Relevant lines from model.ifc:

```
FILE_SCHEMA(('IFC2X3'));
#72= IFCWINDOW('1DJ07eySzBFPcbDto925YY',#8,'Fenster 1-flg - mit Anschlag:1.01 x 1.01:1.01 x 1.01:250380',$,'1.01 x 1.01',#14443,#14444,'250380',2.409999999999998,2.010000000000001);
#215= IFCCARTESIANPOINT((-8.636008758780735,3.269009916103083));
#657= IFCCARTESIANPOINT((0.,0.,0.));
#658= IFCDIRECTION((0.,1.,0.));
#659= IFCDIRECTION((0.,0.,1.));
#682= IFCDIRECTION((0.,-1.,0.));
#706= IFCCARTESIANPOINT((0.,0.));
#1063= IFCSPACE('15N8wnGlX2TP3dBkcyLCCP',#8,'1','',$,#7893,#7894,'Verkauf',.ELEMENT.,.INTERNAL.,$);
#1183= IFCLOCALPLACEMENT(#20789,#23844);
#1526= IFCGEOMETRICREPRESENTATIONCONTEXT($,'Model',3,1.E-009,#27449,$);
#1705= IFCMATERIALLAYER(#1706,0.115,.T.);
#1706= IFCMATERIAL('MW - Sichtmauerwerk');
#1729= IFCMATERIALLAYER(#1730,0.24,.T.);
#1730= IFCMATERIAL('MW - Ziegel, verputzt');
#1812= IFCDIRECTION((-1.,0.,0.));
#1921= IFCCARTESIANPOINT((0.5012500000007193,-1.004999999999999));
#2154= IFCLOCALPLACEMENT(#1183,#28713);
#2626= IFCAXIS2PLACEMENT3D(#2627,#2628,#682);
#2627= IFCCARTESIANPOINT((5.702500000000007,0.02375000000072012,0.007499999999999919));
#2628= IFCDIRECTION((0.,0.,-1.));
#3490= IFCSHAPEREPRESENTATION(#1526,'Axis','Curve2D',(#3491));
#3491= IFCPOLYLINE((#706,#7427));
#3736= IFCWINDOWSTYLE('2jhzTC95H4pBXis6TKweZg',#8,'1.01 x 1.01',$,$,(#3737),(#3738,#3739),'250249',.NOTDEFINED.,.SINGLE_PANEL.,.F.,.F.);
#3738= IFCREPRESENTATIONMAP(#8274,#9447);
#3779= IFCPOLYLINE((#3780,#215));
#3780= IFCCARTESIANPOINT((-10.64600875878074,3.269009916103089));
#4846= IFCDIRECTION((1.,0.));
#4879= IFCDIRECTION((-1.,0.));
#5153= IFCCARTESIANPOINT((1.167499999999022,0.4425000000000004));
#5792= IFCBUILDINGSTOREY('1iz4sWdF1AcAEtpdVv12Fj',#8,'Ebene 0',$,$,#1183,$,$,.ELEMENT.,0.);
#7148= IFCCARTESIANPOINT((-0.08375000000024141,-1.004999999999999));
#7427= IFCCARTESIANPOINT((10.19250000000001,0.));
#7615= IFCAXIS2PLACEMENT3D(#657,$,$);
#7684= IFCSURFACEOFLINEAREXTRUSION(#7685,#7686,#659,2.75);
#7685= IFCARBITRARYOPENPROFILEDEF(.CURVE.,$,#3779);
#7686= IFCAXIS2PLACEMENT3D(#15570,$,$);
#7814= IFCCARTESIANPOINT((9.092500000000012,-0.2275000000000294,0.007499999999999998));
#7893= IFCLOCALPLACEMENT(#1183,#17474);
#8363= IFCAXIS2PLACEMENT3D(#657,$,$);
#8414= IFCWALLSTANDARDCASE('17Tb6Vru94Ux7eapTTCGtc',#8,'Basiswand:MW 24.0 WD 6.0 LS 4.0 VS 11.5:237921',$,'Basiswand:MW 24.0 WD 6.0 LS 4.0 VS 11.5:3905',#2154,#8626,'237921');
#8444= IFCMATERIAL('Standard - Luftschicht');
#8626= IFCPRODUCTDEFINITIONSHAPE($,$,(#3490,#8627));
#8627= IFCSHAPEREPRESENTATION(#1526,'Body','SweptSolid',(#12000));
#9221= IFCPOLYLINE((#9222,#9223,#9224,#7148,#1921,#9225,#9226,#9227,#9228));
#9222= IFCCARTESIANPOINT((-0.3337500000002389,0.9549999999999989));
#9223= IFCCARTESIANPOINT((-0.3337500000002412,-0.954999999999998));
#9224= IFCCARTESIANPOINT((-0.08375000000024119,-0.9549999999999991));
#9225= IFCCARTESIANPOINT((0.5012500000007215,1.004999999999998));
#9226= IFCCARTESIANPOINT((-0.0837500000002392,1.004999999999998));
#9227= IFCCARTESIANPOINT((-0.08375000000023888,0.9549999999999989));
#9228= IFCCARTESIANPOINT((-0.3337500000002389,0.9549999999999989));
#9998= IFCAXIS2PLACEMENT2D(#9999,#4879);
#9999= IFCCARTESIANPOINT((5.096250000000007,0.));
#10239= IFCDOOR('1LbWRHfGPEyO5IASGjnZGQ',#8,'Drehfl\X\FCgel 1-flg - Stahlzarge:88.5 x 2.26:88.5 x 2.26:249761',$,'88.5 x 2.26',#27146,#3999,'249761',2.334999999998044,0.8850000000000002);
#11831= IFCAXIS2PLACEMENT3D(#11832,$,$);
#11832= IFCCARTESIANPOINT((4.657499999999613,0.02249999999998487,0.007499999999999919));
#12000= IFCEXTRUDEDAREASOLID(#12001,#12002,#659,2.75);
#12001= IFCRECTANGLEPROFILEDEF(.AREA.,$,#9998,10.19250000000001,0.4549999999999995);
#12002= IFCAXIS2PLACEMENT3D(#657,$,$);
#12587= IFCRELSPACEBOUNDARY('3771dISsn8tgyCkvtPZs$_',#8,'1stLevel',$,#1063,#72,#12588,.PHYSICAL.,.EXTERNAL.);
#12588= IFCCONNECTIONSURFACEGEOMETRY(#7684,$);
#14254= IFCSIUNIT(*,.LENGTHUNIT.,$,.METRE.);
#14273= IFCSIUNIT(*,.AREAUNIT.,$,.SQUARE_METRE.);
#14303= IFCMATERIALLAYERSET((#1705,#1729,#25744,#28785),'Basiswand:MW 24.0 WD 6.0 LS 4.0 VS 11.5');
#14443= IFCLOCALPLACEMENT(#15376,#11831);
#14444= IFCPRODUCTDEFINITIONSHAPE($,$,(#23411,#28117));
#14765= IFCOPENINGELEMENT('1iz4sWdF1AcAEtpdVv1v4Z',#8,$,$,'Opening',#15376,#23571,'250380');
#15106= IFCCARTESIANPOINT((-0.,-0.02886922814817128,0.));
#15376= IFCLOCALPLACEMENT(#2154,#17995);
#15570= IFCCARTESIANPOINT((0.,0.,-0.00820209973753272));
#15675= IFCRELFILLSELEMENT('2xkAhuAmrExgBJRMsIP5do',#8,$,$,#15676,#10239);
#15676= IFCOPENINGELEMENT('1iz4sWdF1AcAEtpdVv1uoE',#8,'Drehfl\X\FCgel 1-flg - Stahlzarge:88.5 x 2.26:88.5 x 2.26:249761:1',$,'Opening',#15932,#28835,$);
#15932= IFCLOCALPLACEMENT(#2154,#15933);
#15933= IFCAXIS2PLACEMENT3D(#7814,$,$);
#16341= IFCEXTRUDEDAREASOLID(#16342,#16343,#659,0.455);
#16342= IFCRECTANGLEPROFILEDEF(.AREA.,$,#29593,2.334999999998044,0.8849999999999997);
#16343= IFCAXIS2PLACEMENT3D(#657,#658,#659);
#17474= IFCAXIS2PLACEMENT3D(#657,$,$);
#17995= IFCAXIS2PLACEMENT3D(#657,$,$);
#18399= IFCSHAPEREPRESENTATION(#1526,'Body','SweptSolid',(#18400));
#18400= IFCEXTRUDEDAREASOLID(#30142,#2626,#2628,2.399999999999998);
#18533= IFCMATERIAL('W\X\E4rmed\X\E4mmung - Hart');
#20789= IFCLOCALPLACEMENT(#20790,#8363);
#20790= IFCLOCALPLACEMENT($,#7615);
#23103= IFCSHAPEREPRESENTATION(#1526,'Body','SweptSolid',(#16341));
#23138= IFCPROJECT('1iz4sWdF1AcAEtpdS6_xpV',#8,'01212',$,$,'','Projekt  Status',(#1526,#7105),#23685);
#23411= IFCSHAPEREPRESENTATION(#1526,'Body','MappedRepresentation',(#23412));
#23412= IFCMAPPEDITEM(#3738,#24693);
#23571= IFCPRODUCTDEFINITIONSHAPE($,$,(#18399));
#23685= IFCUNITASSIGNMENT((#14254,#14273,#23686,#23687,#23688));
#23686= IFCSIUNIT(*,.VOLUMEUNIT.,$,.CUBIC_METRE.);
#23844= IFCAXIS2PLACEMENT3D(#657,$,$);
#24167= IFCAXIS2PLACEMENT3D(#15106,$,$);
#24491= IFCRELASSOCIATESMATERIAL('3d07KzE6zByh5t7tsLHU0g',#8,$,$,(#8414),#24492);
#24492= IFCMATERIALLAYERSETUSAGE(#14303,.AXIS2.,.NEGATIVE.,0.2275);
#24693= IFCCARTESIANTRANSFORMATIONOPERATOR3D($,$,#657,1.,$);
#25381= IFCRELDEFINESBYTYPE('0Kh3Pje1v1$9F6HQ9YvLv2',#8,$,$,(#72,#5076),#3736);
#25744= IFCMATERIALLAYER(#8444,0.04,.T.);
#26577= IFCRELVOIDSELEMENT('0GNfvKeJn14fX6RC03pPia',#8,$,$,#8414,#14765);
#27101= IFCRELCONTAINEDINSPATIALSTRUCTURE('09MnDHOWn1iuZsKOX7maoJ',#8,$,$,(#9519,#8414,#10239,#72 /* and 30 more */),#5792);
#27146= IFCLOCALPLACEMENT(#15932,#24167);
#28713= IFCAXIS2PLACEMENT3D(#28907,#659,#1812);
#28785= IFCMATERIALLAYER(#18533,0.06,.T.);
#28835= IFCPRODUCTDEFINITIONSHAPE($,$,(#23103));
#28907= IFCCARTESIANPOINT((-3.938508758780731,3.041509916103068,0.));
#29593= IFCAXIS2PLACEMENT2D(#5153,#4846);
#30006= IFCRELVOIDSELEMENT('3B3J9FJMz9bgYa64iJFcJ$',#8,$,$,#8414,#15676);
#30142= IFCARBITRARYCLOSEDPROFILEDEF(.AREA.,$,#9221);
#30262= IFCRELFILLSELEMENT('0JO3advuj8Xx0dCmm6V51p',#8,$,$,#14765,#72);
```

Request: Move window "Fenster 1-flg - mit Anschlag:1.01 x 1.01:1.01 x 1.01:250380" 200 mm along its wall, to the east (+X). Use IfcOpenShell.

```python
import numpy as np
import ifcopenshell
import ifcopenshell.api.geometry
import ifcopenshell.util.placement
import ifcopenshell.util.unit

model = ifcopenshell.open("model.ifc")
unit_scale = ifcopenshell.util.unit.calculate_unit_scale(model)

window = model.by_id(72)
opening = window.FillsVoids[0].RelatingOpeningElement
wall = opening.VoidsElements[0].RelatingBuildingElement

wall_matrix = ifcopenshell.util.placement.get_local_placement(wall.ObjectPlacement)
shift = wall_matrix[:3, 0] * -0.2 / unit_scale
before = ifcopenshell.util.placement.get_local_placement(window.ObjectPlacement)[:3, 3].copy()

# The window is placed relative to its opening, so it follows when the opening moves.
matrix = ifcopenshell.util.placement.get_local_placement(opening.ObjectPlacement)
matrix[:3, 3] += shift
ifcopenshell.api.geometry.edit_object_placement(
    model, product=opening, matrix=matrix, is_si=False, should_transform_children=True
)

# Space boundary surfaces are stored in each space's coordinates; move them too.
for rel in window.ProvidesBoundaries:
    if not rel.ConnectionGeometry:
        continue
    surface = rel.ConnectionGeometry.SurfaceOnRelatingElement
    space_matrix = ifcopenshell.util.placement.get_local_placement(rel.RelatingSpace.ObjectPlacement)
    point = np.array(surface.Position.Location.Coordinates) + space_matrix[:3, :3].T @ shift
    surface.Position = model.createIfcAxis2Placement3D(
        model.createIfcCartesianPoint(point.tolist()), surface.Position.Axis, surface.Position.RefDirection
    )

after = ifcopenshell.util.placement.get_local_placement(window.ObjectPlacement)[:3, 3]
print("window moved by", (after - before).round(3) + 0.0)

model.write("model_v2.ifc")
```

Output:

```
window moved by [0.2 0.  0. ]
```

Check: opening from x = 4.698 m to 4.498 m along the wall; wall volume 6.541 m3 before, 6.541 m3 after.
